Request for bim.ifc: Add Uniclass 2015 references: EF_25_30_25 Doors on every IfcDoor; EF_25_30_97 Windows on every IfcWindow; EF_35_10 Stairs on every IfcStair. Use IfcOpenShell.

First a look at what the model holds.

```python
import ifcopenshell

model = ifcopenshell.open("bim.ifc")
print(model.schema)
print("classifications:", [c.Name for c in model.by_type("IfcClassification")])
for ifc_class in ("IfcDoor", "IfcRoof", "IfcStair", "IfcWall", "IfcWindow"):
    print(ifc_class, len(model.by_type(ifc_class)))
```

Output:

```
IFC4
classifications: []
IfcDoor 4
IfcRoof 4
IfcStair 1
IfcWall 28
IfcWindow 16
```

```python
import ifcopenshell
import ifcopenshell.api.classification

model = ifcopenshell.open("bim.ifc")

system = ifcopenshell.api.classification.add_classification(model, classification="Uniclass 2015")

codes = {
    "IfcDoor": ("EF_25_30_25", "Doors"),
    "IfcWindow": ("EF_25_30_97", "Windows"),
    "IfcStair": ("EF_35_10", "Stairs"),
}
for ifc_class, (code, name) in codes.items():
    products = model.by_type(ifc_class)
    ifcopenshell.api.classification.add_reference(
        model, products=products, classification=system, identification=code, name=name
    )
    print(code, len(products))

model.write("bim_edited.ifc")
```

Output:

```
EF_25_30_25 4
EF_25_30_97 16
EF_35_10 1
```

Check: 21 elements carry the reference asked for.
